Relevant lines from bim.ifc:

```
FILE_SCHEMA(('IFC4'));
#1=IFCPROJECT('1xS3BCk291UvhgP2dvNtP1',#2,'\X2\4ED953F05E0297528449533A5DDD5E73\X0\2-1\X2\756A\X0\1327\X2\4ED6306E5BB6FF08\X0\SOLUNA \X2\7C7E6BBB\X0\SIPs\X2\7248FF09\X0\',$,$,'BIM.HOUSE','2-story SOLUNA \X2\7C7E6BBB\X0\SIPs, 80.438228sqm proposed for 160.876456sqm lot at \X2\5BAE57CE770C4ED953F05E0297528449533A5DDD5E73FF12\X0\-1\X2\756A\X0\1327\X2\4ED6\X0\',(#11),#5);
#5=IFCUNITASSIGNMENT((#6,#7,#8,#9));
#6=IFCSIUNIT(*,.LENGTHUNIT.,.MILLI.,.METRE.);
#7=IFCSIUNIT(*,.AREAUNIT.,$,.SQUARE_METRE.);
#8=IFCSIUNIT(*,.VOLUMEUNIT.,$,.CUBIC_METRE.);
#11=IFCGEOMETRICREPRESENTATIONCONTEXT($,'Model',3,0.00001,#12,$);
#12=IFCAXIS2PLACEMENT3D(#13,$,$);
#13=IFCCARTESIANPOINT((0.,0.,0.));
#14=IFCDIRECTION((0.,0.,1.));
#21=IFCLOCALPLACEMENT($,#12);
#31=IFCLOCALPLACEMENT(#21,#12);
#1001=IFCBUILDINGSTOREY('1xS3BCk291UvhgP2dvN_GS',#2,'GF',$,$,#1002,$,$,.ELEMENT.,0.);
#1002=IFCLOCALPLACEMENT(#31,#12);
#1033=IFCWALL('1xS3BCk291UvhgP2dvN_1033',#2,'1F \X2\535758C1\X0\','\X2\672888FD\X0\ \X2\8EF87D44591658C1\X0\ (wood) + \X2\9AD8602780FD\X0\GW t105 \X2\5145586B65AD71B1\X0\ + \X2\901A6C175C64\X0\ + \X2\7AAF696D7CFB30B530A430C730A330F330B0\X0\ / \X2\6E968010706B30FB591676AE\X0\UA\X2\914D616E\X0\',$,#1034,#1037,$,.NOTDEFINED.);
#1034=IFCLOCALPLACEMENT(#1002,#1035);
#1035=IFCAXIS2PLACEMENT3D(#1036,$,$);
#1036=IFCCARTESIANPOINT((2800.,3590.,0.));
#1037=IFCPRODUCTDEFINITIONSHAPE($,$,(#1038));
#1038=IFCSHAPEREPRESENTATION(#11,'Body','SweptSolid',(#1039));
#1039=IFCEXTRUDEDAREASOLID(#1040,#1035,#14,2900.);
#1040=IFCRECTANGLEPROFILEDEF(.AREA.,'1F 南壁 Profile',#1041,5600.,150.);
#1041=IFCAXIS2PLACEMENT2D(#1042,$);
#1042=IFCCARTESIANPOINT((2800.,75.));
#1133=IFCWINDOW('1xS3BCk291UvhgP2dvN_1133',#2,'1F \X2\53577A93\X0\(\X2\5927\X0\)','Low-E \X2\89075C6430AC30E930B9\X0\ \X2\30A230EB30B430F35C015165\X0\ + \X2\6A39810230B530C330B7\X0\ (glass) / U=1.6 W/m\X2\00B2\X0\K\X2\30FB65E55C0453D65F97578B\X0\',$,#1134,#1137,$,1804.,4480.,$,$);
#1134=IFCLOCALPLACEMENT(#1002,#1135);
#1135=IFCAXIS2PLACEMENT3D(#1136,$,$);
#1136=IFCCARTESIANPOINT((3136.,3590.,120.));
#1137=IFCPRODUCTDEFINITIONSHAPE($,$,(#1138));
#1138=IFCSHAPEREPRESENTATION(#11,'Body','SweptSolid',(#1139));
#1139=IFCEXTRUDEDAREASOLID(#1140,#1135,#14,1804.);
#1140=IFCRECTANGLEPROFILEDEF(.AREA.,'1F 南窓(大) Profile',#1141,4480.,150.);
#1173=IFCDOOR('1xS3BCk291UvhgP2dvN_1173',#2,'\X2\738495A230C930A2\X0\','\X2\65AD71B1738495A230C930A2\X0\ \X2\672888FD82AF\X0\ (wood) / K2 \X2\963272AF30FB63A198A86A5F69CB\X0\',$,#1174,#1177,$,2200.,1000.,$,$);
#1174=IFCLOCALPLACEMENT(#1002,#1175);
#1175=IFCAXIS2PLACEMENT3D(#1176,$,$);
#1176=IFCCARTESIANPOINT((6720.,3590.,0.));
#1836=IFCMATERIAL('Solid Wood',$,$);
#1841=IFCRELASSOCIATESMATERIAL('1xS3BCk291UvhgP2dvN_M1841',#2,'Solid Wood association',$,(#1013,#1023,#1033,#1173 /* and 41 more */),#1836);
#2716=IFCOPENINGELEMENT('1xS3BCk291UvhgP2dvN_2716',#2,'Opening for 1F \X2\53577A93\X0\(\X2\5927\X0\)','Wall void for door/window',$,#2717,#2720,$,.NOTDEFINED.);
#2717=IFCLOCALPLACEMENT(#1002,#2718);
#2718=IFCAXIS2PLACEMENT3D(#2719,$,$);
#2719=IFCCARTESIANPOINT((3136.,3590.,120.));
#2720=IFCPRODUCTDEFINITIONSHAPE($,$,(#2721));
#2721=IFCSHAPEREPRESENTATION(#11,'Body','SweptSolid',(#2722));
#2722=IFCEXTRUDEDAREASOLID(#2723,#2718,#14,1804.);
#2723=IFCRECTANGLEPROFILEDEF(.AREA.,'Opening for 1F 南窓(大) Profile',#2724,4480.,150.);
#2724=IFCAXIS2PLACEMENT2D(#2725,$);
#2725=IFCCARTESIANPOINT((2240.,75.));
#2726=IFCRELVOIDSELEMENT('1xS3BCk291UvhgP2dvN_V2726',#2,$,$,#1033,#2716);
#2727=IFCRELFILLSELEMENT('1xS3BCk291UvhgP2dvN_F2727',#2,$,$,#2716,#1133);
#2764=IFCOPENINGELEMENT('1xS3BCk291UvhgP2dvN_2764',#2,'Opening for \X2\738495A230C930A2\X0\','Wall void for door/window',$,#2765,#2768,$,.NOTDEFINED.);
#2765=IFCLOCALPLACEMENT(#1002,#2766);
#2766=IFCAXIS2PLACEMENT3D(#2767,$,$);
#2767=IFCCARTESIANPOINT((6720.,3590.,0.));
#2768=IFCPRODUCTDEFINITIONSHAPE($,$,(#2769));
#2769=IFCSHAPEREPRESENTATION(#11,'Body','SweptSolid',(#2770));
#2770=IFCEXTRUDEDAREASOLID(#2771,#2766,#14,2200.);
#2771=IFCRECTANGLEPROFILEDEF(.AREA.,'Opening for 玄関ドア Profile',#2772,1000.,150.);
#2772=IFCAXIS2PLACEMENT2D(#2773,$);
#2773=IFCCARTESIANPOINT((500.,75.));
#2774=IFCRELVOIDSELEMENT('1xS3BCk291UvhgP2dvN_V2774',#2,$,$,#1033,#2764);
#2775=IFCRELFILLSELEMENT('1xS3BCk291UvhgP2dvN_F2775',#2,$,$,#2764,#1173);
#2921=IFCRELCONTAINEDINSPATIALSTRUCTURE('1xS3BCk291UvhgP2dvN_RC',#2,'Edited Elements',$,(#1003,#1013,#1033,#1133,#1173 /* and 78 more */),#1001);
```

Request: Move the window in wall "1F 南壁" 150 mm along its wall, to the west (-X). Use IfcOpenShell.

```python
import ifcopenshell
import ifcopenshell.api.geometry
import ifcopenshell.util.placement
import ifcopenshell.util.unit

model = ifcopenshell.open("bim.ifc")
unit_scale = ifcopenshell.util.unit.calculate_unit_scale(model)

window = model.by_guid("1xS3BCk291UvhgP2dvN_1133")
opening = window.FillsVoids[0].RelatingOpeningElement
wall = opening.VoidsElements[0].RelatingBuildingElement

wall_matrix = ifcopenshell.util.placement.get_local_placement(wall.ObjectPlacement)
shift = wall_matrix[:3, 0] * -0.15 / unit_scale
before = ifcopenshell.util.placement.get_local_placement(window.ObjectPlacement)[:3, 3].copy()

# The window is not placed relative to its opening, so move both.
for product in (opening, window):
    matrix = ifcopenshell.util.placement.get_local_placement(product.ObjectPlacement)
    matrix[:3, 3] += shift
    ifcopenshell.api.geometry.edit_object_placement(model, product=product, matrix=matrix, is_si=False)

after = ifcopenshell.util.placement.get_local_placement(window.ObjectPlacement)[:3, 3]
print("window moved by", (after - before).round(3) + 0.0)

model.write("bim_v2.ifc")
```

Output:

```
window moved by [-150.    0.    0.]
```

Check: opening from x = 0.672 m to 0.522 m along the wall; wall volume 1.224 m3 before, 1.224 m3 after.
